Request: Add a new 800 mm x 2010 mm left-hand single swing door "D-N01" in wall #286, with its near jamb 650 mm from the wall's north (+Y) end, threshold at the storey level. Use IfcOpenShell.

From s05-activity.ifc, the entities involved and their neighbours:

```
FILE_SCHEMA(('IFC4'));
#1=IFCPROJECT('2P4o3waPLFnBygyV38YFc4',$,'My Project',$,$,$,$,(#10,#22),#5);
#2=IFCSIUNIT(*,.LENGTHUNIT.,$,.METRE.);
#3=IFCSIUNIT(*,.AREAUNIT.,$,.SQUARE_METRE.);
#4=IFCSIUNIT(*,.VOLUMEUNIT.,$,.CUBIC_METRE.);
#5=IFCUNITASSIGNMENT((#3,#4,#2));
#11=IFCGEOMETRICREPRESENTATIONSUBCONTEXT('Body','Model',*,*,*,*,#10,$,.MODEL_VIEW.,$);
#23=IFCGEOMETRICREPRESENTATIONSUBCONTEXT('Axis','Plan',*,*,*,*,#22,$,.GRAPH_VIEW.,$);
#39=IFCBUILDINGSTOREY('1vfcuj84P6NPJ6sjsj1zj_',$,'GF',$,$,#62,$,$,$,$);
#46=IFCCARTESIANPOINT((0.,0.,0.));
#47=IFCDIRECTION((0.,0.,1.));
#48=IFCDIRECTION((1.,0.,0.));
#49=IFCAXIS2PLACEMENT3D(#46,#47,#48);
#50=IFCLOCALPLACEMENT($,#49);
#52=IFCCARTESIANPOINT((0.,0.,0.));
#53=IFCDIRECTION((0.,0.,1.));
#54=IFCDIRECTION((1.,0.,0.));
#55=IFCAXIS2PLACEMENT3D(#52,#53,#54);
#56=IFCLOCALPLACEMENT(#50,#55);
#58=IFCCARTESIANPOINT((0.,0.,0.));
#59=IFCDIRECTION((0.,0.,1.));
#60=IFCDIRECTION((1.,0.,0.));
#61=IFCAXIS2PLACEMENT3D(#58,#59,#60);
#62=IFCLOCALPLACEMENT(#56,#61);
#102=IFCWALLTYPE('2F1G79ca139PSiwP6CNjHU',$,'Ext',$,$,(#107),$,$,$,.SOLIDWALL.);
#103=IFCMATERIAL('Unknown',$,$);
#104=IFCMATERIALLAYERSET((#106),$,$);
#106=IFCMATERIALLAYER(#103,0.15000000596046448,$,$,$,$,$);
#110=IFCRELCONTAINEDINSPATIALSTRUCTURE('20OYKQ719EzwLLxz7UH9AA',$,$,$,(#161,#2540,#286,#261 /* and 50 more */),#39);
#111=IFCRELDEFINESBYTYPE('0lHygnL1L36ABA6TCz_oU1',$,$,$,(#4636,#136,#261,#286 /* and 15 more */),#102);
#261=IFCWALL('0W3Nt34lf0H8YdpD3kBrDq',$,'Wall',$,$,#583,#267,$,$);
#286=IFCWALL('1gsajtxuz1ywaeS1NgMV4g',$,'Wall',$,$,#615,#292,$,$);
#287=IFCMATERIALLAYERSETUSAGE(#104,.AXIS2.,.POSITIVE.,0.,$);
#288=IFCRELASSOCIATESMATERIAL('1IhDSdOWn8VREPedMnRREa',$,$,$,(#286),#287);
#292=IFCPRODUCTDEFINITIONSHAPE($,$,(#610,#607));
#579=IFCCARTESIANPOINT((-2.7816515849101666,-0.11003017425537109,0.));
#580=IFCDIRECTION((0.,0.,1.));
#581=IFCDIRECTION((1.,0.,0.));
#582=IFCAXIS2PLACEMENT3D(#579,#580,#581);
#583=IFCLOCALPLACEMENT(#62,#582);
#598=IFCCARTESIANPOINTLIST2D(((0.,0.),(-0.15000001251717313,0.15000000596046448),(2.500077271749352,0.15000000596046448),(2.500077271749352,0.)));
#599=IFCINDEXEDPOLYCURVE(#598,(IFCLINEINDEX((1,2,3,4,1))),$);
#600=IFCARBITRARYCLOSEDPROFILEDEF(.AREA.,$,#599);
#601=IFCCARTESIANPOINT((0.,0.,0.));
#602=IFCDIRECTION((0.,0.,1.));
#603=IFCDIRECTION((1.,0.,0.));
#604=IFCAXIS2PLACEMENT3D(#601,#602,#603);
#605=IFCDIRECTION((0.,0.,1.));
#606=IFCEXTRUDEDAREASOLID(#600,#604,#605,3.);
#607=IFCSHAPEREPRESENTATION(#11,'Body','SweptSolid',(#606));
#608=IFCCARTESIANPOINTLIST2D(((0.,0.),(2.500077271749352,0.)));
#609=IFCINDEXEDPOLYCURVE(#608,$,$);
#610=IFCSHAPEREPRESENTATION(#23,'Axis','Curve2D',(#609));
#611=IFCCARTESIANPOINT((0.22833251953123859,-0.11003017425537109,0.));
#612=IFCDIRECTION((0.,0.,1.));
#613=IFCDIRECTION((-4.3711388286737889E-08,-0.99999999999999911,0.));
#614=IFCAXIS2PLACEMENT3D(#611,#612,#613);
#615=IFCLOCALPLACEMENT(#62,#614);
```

```python
import numpy as np
import ifcopenshell
import ifcopenshell.api.feature
import ifcopenshell.api.geometry
import ifcopenshell.api.root
import ifcopenshell.api.spatial
import ifcopenshell.geom
import ifcopenshell.util.element
import ifcopenshell.util.placement
import ifcopenshell.util.representation
import ifcopenshell.util.shape
import ifcopenshell.util.unit

model = ifcopenshell.open("s05-activity.ifc")
unit_scale = ifcopenshell.util.unit.calculate_unit_scale(model)
settings = ifcopenshell.geom.settings()


def volume(element):
    """Net volume in cubic metres, openings subtracted."""
    shape = ifcopenshell.geom.create_shape(settings, element)
    return ifcopenshell.util.shape.get_volume(shape.geometry)


wall = model.by_id(286)
storey = ifcopenshell.util.element.get_container(wall, ifc_class="IfcBuildingStorey")
context = ifcopenshell.util.representation.get_context(model, "Model", "Body", "MODEL_VIEW")
before = volume(wall)

width, height, from_end, sill = 0.8, 2.01, 0.65, 0.0  # metres

# The wall runs along its own X axis, and the end named is its -X end.
wall_shape = ifcopenshell.geom.create_shape(settings, wall)
x, y, z = ifcopenshell.util.shape.get_vertices(wall_shape.geometry).T
start = x.min() + from_end
face, thickness = float(y.min()), float(y.max() - y.min())
wall_matrix = ifcopenshell.util.placement.get_local_placement(wall.ObjectPlacement)
level = ifcopenshell.util.placement.get_local_placement(storey.ObjectPlacement)[2, 3]


def in_wall(x, y):
    """Placement at x, y metres in the wall's axes, at sill height."""
    matrix = wall_matrix.copy()
    matrix[:, 3] = wall_matrix @ np.array([x / unit_scale, y / unit_scale, 0.0, 1.0])
    matrix[2, 3] = level + sill / unit_scale
    return matrix


# Opening: a box that overshoots both wall faces by 50 mm.
opening = ifcopenshell.api.root.create_entity(model, ifc_class="IfcOpeningElement", predefined_type="OPENING")
box = ifcopenshell.api.geometry.add_wall_representation(
    model, context=context, length=width, height=height, thickness=thickness + 0.1
)
ifcopenshell.api.geometry.assign_representation(model, product=opening, representation=box)
ifcopenshell.api.geometry.edit_object_placement(model, product=opening, matrix=in_wall(start, face - 0.05), is_si=False)
ifcopenshell.api.feature.add_feature(model, feature=opening, element=wall)

door = ifcopenshell.api.root.create_entity(model, ifc_class="IfcDoor", name="D-N01", predefined_type="DOOR")
door.OverallWidth, door.OverallHeight = width / unit_scale, height / unit_scale
door.OperationType = "SINGLE_SWING_LEFT"
body = ifcopenshell.api.geometry.add_door_representation(
    model,
    context=context,
    overall_width=door.OverallWidth,
    overall_height=door.OverallHeight,
    operation_type="SINGLE_SWING_LEFT",
    lining_properties={"LiningDepth": thickness / unit_scale, "ThresholdDepth": thickness / unit_scale},
)
ifcopenshell.api.geometry.assign_representation(model, product=door, representation=body)
ifcopenshell.api.spatial.assign_container(model, products=[door], relating_structure=storey)
ifcopenshell.api.feature.add_filling(model, opening=opening, element=door)

# The lining spans the wall, so the door starts at the wall face.
ifcopenshell.api.geometry.edit_object_placement(model, product=door, matrix=in_wall(start, face), is_si=False)

after = volume(wall)

print(f"wall volume {before:.3f} -> {after:.3f} m3")

model.write("s05-activity_updated.ifc")
```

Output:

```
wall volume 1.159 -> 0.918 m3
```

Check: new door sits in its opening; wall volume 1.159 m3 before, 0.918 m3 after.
